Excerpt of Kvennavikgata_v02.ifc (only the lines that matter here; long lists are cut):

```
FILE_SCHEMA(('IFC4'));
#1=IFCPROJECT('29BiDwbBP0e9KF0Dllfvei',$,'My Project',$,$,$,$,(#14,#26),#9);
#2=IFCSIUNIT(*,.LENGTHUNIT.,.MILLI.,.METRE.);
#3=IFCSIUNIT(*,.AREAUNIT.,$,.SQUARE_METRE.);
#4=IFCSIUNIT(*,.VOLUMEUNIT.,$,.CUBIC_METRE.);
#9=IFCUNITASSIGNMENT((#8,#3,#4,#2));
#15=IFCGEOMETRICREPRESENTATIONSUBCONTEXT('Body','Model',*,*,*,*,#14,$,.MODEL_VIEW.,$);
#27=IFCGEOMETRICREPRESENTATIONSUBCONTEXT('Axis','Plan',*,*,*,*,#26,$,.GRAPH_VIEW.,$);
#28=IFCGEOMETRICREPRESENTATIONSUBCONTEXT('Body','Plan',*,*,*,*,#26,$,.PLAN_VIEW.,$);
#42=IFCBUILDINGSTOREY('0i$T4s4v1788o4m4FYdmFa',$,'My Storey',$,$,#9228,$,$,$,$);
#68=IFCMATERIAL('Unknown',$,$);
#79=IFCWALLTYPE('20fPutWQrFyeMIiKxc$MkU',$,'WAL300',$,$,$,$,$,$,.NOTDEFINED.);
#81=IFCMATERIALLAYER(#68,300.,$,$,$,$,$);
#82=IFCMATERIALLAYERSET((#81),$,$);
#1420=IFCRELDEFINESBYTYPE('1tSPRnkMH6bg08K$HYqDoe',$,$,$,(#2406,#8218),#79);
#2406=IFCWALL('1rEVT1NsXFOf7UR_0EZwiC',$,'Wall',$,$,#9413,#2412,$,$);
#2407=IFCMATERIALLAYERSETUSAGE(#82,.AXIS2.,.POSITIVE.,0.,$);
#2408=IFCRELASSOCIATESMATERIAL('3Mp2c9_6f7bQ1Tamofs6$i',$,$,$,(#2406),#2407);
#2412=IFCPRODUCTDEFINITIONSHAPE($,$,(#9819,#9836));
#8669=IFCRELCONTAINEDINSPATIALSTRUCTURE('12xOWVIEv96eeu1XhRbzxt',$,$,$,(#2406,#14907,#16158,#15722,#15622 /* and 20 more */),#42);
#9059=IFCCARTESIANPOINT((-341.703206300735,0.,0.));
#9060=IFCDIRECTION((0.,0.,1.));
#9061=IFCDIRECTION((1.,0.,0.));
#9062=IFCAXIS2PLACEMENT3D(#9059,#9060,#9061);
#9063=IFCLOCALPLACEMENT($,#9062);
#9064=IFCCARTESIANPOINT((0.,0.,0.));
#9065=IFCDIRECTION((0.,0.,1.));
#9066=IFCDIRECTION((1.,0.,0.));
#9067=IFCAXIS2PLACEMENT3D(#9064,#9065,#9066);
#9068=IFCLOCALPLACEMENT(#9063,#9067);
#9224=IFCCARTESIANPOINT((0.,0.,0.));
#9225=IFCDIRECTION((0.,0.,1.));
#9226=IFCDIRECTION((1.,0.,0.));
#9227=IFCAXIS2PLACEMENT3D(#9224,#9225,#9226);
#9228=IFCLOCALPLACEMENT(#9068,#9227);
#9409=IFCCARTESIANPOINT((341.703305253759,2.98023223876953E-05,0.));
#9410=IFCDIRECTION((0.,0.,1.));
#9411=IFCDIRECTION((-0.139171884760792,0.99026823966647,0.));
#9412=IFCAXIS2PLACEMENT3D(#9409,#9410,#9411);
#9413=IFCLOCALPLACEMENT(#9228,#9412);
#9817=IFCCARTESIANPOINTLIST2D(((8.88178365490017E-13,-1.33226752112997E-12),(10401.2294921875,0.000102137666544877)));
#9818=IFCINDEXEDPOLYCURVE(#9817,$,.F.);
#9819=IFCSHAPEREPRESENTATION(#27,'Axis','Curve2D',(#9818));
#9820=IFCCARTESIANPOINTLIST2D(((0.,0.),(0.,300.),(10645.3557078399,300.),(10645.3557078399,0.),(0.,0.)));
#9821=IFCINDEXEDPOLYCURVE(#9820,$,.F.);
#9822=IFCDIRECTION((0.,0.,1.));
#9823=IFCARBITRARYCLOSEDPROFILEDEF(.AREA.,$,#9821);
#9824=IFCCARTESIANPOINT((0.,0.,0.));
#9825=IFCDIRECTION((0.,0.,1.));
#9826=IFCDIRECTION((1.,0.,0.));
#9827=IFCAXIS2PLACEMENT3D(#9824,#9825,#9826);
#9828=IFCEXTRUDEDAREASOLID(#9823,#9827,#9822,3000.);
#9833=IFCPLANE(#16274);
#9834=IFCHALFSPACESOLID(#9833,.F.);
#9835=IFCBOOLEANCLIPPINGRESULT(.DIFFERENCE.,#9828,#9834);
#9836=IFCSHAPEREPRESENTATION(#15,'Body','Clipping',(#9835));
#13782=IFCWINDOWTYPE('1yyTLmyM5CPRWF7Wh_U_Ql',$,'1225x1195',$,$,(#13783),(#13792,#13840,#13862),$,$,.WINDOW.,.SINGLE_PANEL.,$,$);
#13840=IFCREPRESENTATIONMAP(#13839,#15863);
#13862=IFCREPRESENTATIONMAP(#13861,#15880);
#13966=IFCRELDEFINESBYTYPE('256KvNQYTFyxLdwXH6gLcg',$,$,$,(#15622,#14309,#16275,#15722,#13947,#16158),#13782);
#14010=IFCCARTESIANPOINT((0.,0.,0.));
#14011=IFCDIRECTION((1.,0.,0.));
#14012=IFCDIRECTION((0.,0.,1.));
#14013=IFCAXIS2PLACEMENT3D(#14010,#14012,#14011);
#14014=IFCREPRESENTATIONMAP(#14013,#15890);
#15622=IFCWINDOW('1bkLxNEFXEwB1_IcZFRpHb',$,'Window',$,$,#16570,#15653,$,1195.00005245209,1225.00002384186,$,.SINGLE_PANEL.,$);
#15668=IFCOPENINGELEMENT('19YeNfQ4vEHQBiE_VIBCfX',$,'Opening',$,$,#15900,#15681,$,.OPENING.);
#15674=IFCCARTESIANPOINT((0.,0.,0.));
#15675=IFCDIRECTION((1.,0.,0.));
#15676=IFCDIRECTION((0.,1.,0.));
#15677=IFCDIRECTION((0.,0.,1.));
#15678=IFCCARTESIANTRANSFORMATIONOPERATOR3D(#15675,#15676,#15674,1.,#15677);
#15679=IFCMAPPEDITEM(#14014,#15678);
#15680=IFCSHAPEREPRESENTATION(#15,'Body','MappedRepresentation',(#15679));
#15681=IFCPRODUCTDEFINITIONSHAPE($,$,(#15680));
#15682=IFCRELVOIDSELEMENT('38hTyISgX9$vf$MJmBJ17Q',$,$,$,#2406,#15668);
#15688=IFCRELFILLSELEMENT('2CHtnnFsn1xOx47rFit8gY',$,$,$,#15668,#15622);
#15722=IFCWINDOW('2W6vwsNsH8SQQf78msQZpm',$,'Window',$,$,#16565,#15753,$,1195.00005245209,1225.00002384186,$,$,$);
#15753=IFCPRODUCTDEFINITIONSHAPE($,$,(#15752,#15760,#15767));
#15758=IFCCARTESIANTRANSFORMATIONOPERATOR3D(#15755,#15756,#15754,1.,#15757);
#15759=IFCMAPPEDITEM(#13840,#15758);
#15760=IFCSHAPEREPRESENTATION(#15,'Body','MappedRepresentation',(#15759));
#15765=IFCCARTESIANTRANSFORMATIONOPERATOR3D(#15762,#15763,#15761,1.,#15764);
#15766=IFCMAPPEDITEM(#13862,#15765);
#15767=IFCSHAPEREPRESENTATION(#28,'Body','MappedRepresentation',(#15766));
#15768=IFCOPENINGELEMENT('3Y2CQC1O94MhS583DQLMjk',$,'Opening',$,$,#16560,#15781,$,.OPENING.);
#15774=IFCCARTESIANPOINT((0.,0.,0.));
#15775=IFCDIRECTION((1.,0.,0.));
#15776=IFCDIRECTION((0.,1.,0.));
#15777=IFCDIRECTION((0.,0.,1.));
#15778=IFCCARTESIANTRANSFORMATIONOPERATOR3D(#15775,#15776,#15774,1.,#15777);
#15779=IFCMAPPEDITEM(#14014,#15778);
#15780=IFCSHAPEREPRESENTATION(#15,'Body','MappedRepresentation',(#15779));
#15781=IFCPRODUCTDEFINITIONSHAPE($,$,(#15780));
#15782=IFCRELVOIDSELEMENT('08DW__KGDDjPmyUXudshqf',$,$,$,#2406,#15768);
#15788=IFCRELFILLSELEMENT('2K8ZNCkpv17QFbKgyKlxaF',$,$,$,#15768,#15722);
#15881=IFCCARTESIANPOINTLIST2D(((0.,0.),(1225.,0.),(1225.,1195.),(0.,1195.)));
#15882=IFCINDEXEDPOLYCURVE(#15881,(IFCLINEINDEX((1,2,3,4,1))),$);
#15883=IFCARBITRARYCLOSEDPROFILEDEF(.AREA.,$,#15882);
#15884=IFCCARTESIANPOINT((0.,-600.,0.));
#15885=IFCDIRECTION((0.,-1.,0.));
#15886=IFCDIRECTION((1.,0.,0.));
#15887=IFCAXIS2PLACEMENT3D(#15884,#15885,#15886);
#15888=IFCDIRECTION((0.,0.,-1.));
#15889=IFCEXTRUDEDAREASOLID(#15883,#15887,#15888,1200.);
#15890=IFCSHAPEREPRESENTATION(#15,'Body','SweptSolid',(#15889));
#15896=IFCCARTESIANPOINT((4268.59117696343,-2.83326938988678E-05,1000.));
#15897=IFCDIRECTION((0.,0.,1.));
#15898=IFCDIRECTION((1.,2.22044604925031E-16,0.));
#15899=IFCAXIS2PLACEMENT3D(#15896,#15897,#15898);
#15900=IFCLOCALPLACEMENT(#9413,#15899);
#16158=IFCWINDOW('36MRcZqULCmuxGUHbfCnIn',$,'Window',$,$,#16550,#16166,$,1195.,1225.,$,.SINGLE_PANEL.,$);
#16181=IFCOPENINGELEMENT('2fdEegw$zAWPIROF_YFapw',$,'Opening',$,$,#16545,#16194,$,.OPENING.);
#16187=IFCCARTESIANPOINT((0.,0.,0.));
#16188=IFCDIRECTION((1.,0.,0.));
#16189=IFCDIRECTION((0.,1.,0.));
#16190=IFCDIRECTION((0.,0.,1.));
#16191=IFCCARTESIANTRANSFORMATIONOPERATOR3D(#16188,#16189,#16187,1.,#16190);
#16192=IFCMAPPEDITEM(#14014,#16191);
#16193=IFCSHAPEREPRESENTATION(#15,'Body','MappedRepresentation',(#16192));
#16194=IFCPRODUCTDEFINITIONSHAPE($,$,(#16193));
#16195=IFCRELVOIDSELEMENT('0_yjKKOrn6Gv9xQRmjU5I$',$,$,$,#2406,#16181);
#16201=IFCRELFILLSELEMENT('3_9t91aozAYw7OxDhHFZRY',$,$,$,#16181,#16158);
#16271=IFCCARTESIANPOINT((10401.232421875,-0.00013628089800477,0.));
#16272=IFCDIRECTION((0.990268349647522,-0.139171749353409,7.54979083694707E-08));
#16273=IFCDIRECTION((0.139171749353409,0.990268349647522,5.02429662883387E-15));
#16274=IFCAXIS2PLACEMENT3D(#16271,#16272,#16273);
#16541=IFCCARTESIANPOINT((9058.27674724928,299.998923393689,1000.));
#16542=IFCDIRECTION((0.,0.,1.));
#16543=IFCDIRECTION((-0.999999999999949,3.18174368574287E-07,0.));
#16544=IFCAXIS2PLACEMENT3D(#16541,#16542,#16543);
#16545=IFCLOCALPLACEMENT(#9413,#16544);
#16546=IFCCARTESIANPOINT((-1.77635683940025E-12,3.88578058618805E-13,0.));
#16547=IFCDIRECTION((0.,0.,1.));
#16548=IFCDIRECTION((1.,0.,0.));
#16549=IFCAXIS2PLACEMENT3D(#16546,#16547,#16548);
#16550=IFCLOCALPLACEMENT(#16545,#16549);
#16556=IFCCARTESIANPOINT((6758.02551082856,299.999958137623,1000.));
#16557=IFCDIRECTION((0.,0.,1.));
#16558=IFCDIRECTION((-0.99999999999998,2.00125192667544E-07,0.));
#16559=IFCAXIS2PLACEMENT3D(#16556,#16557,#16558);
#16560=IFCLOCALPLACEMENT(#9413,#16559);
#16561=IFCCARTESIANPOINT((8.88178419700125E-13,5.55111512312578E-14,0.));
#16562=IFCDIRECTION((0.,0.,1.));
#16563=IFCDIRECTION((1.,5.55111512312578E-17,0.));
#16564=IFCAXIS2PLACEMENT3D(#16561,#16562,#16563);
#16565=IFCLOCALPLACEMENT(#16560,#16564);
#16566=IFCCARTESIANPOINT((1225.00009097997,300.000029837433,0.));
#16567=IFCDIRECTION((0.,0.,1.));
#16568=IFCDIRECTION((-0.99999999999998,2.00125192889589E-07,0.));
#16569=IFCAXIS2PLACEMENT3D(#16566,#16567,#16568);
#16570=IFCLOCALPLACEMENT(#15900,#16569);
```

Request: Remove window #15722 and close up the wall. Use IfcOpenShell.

```python
import ifcopenshell
import ifcopenshell.api.feature
import ifcopenshell.api.root
import ifcopenshell.geom
import ifcopenshell.util.shape

model = ifcopenshell.open("Kvennavikgata_v02.ifc")
settings = ifcopenshell.geom.settings()


def volume(element):
    """Net volume in cubic metres, openings subtracted."""
    shape = ifcopenshell.geom.create_shape(settings, element)
    return ifcopenshell.util.shape.get_volume(shape.geometry)


window = model.by_guid("2W6vwsNsH8SQQf78msQZpm")
opening = window.FillsVoids[0].RelatingOpeningElement
wall = opening.VoidsElements[0].RelatingBuildingElement
before = volume(wall)

ifcopenshell.api.root.remove_product(model, product=window)
ifcopenshell.api.feature.remove_feature(model, feature=opening)

after = volume(wall)

print(f"wall volume {before:.3f} -> {after:.3f} m3")

model.write("Kvennavikgata_v02_edited.ifc")
```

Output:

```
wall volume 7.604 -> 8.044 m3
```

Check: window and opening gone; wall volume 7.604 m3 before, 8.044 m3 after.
